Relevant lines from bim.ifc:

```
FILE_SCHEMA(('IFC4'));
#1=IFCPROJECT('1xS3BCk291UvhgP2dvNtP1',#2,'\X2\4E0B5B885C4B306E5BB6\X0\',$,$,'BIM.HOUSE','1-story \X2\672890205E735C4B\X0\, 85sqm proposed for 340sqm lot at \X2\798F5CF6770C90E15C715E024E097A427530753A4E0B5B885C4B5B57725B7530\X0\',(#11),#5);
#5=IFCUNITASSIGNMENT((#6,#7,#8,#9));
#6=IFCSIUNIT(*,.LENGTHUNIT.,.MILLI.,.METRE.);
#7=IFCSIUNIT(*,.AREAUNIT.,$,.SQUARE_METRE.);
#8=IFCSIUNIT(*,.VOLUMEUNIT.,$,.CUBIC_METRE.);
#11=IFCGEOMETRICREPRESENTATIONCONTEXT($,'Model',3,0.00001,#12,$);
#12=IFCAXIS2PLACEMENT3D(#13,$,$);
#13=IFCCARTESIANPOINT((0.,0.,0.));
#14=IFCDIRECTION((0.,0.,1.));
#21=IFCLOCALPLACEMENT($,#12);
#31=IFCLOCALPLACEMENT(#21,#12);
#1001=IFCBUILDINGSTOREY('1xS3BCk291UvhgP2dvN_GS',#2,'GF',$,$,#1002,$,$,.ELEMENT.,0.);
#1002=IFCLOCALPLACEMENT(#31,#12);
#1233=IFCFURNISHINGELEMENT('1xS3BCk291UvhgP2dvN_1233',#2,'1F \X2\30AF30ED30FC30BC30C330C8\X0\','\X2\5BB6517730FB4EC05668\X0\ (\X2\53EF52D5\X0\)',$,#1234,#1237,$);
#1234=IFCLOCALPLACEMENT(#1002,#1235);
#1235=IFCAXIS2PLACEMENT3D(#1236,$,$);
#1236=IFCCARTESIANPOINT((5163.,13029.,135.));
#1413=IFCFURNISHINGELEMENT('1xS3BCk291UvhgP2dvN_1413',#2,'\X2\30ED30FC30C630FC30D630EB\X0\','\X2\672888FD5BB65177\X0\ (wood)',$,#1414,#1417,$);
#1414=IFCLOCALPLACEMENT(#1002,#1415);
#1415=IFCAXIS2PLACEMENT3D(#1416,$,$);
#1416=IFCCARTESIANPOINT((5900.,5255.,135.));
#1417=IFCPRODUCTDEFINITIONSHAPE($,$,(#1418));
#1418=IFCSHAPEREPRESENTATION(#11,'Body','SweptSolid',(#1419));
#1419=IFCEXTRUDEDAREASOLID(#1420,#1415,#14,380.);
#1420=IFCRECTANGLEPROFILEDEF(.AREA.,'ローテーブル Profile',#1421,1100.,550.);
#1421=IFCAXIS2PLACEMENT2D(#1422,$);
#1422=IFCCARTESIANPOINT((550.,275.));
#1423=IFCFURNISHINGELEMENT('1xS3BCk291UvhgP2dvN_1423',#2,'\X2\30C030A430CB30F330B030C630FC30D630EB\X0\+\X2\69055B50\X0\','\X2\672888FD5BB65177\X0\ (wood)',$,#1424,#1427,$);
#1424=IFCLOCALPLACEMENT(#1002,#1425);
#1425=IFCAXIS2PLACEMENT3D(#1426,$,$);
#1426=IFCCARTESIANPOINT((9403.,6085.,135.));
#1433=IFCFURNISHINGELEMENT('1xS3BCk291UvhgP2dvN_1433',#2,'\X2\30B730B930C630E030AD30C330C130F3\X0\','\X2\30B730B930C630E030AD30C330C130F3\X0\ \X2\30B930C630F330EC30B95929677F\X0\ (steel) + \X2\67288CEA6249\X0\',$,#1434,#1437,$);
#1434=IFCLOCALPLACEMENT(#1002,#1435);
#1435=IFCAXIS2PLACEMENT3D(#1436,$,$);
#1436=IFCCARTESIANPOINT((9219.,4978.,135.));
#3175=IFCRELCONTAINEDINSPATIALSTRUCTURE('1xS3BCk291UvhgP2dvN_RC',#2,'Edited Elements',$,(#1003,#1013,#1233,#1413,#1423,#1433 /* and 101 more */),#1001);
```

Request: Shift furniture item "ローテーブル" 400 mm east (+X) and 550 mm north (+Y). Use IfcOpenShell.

```python
import ifcopenshell
import ifcopenshell.api.geometry
import ifcopenshell.util.placement
import ifcopenshell.util.unit

model = ifcopenshell.open("bim.ifc")
unit_scale = ifcopenshell.util.unit.calculate_unit_scale(model)

item = model.by_guid("1xS3BCk291UvhgP2dvN_1413")
matrix = ifcopenshell.util.placement.get_local_placement(item.ObjectPlacement)
matrix[0, 3] += 0.4 / unit_scale
matrix[1, 3] += 0.55 / unit_scale
ifcopenshell.api.geometry.edit_object_placement(model, product=item, matrix=matrix, is_si=False)

print(ifcopenshell.util.placement.get_local_placement(item.ObjectPlacement).round(3) + 0.0)

model.write("bim_v2.ifc")
```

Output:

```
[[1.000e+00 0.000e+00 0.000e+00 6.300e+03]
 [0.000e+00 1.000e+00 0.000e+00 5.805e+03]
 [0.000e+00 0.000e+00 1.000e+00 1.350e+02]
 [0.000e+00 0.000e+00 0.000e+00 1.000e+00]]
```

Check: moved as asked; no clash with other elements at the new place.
